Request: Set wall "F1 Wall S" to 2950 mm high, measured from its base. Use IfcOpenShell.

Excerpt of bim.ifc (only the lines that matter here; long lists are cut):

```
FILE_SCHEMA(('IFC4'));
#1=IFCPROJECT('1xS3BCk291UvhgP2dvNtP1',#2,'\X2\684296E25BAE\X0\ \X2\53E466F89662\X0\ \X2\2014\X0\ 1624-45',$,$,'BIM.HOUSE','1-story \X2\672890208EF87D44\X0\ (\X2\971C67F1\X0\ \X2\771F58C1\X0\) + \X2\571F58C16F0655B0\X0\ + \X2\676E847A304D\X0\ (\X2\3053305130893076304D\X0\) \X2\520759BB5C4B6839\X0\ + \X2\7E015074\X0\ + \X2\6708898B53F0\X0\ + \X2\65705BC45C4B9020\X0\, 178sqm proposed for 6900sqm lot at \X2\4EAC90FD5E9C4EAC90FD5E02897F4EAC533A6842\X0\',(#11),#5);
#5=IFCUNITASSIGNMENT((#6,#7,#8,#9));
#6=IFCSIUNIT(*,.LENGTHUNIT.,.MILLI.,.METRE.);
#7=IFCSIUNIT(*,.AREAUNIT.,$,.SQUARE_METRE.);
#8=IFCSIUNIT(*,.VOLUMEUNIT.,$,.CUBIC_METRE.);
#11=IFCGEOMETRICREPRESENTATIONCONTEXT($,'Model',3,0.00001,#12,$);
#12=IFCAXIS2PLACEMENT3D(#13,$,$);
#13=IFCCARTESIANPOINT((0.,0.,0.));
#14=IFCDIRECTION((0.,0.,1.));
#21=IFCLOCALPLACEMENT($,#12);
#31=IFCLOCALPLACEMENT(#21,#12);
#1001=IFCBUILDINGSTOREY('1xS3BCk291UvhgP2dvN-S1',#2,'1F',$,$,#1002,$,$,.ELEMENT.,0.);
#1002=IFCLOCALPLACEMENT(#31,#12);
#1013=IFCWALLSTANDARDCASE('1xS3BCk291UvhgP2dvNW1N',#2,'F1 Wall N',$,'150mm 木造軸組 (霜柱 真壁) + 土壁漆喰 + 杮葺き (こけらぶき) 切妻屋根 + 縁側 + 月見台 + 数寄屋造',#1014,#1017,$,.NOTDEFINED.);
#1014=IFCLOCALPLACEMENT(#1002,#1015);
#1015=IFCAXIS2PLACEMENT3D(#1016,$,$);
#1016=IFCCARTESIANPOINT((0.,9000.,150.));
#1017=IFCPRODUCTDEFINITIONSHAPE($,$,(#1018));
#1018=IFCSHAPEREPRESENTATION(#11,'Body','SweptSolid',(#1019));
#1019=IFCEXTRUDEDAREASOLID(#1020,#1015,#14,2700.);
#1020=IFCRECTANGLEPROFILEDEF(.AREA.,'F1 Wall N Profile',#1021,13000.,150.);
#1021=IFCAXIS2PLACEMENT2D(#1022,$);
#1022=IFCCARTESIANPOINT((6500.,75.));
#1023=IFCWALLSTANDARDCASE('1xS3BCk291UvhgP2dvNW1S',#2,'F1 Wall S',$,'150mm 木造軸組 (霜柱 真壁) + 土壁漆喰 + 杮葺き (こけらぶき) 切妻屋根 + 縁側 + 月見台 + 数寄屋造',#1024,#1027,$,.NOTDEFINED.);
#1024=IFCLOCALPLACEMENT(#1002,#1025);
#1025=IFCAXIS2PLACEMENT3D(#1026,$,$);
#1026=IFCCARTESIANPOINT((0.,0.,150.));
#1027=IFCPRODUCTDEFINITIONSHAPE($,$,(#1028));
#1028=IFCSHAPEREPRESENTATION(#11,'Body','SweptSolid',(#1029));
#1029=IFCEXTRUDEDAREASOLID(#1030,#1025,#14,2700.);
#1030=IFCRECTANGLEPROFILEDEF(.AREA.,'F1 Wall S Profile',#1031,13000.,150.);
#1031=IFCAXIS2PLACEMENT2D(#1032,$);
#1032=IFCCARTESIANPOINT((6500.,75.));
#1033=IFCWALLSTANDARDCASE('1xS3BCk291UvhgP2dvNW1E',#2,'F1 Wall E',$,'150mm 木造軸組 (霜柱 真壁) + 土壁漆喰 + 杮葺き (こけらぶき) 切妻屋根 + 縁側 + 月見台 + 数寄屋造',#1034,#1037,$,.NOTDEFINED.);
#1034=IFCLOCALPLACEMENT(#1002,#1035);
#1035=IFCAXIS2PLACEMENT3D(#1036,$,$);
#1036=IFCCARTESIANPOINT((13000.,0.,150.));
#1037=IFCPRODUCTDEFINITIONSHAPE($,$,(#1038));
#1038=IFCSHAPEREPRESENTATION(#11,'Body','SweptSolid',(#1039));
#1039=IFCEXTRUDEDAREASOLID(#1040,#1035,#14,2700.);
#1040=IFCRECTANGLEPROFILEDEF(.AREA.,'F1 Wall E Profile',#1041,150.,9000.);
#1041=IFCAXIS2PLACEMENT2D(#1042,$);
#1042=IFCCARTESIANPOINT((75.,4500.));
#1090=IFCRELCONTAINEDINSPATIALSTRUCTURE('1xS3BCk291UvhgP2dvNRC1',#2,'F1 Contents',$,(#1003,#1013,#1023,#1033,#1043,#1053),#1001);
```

```python
import ifcopenshell
import ifcopenshell.geom
import ifcopenshell.util.shape
import ifcopenshell.util.unit

model = ifcopenshell.open("bim.ifc")
unit_scale = ifcopenshell.util.unit.calculate_unit_scale(model)
settings = ifcopenshell.geom.settings()


def volume(element):
    """Net volume in cubic metres, openings subtracted."""
    shape = ifcopenshell.geom.create_shape(settings, element)
    return ifcopenshell.util.shape.get_volume(shape.geometry)


wall = model.by_guid("1xS3BCk291UvhgP2dvNW1S")
before = volume(wall)

body = next(r for r in wall.Representation.Representations if r.RepresentationIdentifier == "Body")
solid = body.Items[0]
old_height = solid.Depth
solid.Depth = 2.95 / unit_scale
after = volume(wall)

print(f"height {old_height:g} -> {solid.Depth:g}, volume {before:.3f} -> {after:.3f} m3")

model.write("bim-out.ifc")
```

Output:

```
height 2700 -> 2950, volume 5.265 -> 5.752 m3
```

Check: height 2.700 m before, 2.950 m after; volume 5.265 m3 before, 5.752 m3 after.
